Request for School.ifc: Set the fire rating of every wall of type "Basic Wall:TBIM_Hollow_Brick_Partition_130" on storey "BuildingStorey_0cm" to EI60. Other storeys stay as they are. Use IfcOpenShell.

First a look at what the model holds.

```python
import ifcopenshell
import ifcopenshell.util.element

model = ifcopenshell.open("School.ifc")
print(model.schema)
storey = next(s for s in model.by_type("IfcBuildingStorey") if s.Name == "BuildingStorey_0cm")
walls = [e for e in ifcopenshell.util.element.get_decomposition(storey) if e.is_a("IfcWall")]
seen = {}
for e in walls:
    element_type = ifcopenshell.util.element.get_type(e)
    key = (element_type.Name if element_type != e and element_type else None, ifcopenshell.util.element.get_pset(e, "Pset_WallCommon", "FireRating"))
    seen[key] = seen.get(key, 0) + 1
for (name, value), count in sorted(seen.items(), key=str):
    print(count, "x", name, "|", value)
```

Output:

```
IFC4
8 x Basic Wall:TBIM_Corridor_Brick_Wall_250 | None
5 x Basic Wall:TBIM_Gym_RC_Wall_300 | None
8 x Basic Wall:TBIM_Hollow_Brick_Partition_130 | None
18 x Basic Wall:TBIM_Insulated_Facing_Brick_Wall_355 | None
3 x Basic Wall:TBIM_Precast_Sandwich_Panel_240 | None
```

```python
import ifcopenshell
import ifcopenshell.api.pset
import ifcopenshell.util.element

model = ifcopenshell.open("School.ifc")

storey = next(s for s in model.by_type("IfcBuildingStorey") if s.Name == "BuildingStorey_0cm")
walls = [e for e in ifcopenshell.util.element.get_decomposition(storey) if e.is_a("IfcWall")]

count = 0
for e in walls:
    element_type = ifcopenshell.util.element.get_type(e)
    if element_type in (None, e) or element_type.Name != "Basic Wall:TBIM_Hollow_Brick_Partition_130":
        continue
    # add_pset returns the element's existing set when there is one.
    pset = ifcopenshell.api.pset.add_pset(model, product=e, name="Pset_WallCommon")
    ifcopenshell.api.pset.edit_pset(model, pset=pset, properties={"FireRating": "EI60"})
    count += 1

print(count, "walls updated")

model.write("School_v2.ifc")
```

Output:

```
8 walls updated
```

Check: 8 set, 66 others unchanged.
